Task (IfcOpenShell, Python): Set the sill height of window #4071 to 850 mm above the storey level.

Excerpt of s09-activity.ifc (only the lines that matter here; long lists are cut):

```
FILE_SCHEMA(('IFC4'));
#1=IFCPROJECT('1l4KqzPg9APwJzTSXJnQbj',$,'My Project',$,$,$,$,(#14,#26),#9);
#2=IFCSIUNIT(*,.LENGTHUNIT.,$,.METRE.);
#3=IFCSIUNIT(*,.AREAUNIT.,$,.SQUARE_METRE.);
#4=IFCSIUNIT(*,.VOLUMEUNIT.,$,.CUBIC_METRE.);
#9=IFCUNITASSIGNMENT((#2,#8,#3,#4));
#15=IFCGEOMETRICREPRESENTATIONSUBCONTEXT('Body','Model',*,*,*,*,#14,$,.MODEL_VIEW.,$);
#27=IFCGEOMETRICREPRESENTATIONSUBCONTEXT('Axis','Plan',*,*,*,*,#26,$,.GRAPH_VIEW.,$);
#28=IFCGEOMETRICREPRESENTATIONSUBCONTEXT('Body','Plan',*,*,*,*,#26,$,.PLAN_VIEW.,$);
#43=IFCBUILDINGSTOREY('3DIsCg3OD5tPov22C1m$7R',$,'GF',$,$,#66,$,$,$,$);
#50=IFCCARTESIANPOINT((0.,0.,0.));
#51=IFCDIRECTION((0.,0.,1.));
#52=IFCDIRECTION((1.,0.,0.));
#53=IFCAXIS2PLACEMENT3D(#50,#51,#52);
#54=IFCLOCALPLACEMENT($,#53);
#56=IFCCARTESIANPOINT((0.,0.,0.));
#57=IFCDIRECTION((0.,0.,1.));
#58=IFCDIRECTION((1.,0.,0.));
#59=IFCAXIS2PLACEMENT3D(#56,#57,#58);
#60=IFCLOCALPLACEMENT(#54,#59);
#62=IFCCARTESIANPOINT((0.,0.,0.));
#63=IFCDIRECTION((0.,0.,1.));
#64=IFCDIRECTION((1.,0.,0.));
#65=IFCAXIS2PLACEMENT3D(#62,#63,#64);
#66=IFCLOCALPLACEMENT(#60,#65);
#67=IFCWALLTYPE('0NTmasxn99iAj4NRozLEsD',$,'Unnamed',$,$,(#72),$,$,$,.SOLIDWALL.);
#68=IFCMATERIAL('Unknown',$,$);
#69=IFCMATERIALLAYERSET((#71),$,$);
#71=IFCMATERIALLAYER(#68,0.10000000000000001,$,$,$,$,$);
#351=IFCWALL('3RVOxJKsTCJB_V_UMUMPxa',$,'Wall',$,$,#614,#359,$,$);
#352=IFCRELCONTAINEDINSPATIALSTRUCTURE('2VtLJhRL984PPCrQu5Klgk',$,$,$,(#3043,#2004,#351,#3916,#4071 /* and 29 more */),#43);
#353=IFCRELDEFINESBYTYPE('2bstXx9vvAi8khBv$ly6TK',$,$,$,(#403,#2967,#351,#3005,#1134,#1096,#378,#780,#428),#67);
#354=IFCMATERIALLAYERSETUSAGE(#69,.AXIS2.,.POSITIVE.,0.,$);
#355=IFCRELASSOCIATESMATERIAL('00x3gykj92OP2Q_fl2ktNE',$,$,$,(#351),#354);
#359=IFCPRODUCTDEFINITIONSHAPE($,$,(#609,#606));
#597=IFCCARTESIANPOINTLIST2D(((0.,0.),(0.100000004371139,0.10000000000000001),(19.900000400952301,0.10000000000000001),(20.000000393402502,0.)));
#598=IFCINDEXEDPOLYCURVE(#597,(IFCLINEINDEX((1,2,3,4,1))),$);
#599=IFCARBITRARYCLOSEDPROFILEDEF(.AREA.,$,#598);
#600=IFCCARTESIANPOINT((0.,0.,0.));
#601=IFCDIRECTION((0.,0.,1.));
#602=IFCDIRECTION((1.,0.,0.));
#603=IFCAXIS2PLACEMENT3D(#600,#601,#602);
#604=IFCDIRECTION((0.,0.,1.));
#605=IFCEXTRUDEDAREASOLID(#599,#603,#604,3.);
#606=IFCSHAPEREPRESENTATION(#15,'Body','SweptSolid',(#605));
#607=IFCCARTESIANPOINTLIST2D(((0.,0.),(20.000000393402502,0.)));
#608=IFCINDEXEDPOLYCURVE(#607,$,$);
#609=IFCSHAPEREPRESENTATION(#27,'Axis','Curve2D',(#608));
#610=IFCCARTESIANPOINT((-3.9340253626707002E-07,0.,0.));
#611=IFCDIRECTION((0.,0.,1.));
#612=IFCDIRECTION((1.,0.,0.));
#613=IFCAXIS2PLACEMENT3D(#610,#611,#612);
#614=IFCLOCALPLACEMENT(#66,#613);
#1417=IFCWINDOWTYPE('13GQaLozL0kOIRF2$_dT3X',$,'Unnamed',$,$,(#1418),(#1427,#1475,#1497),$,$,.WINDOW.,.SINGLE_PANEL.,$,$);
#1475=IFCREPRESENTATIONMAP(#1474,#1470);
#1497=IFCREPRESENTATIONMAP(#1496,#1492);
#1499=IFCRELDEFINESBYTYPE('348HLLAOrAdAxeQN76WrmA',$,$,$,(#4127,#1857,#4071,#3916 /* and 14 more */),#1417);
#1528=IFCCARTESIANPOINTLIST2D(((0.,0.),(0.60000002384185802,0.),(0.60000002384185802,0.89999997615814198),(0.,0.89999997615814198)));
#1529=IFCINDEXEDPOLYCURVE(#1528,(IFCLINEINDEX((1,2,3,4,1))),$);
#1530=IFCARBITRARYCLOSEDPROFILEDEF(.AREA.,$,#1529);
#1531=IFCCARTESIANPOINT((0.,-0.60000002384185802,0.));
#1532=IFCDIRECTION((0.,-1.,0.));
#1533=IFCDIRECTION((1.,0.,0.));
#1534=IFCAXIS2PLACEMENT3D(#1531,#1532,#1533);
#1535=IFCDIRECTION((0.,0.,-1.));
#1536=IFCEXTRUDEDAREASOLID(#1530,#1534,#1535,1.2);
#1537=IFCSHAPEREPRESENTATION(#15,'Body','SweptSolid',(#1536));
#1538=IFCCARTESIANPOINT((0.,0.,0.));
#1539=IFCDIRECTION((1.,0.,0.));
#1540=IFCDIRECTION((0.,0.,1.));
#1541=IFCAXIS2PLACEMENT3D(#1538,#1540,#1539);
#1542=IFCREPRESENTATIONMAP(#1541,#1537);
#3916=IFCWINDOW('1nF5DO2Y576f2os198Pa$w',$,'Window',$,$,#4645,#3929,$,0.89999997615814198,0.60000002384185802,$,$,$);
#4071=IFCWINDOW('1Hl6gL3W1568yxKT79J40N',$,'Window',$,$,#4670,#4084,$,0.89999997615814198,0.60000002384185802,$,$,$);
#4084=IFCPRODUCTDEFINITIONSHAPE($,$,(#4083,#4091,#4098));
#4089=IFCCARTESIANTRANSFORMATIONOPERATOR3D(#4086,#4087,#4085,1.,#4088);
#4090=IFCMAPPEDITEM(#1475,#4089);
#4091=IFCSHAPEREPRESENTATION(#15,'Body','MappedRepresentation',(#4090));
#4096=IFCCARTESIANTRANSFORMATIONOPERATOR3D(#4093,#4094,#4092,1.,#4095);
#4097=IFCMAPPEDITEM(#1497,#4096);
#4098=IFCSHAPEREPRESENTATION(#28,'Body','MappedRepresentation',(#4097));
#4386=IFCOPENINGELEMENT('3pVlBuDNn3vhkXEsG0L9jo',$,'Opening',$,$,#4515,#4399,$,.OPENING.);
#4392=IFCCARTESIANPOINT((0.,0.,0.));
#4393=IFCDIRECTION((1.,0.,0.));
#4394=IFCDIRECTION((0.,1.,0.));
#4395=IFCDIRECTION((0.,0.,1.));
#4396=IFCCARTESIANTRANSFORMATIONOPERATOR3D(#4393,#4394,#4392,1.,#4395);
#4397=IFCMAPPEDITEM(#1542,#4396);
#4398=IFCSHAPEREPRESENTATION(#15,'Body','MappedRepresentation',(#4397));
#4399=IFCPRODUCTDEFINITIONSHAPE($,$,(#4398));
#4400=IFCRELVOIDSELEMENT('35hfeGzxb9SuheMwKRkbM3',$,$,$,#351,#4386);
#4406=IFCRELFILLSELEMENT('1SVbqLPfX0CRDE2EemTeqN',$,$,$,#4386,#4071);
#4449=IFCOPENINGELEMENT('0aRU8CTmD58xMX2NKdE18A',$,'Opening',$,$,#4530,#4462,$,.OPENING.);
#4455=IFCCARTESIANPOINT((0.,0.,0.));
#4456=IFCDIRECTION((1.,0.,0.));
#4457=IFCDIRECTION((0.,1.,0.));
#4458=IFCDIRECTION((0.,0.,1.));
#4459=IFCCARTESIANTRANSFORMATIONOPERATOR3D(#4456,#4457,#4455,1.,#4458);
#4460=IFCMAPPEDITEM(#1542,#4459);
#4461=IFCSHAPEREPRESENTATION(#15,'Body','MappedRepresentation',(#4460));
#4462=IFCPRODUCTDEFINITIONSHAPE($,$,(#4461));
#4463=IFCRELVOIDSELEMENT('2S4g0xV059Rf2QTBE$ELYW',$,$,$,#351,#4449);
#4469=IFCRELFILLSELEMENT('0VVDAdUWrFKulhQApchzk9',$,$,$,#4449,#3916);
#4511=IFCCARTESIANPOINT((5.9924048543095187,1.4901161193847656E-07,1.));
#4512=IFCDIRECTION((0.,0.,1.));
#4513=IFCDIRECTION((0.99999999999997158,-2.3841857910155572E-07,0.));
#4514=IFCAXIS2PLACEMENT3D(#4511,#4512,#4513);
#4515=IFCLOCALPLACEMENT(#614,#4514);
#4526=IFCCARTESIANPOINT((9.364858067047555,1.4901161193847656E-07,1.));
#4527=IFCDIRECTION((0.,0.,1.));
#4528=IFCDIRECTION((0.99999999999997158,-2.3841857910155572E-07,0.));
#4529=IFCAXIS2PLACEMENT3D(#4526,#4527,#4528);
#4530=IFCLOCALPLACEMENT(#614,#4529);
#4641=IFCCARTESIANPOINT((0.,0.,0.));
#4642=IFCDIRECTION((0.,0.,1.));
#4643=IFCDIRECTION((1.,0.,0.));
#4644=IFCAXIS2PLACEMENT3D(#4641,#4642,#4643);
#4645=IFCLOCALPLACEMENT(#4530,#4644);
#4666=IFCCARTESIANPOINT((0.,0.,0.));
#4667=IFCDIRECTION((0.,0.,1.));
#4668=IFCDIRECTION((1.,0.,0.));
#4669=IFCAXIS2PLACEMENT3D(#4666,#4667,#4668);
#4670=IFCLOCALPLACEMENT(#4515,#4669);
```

```python
import numpy as np
import ifcopenshell
import ifcopenshell.api.geometry
import ifcopenshell.geom
import ifcopenshell.util.element
import ifcopenshell.util.placement
import ifcopenshell.util.shape
import ifcopenshell.util.unit

model = ifcopenshell.open("s09-activity.ifc")
unit_scale = ifcopenshell.util.unit.calculate_unit_scale(model)

window = model.by_guid("1Hl6gL3W1568yxKT79J40N")
opening = window.FillsVoids[0].RelatingOpeningElement
storey = ifcopenshell.util.element.get_container(window, ifc_class="IfcBuildingStorey")
level = ifcopenshell.util.placement.get_local_placement(storey.ObjectPlacement)[2, 3]

# The opening's origin need not be at the sill, so measure its lowest point.
shape = ifcopenshell.geom.create_shape(ifcopenshell.geom.settings(), opening)
bottom = ifcopenshell.util.shape.get_shape_bottom_elevation(shape, shape.geometry) / unit_scale
dz = level + 0.85 - bottom

shift = np.array([0.0, 0.0, dz])
# The window is placed relative to its opening, so it follows when the opening moves.
matrix = ifcopenshell.util.placement.get_local_placement(opening.ObjectPlacement)
matrix[:3, 3] += shift
ifcopenshell.api.geometry.edit_object_placement(
    model, product=opening, matrix=matrix, is_si=False, should_transform_children=True
)

print(f"moved by {dz * unit_scale:+.3f} m")

model.write("s09-activity_edited.ifc")
```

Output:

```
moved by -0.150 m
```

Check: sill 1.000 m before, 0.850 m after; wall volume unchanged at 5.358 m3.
